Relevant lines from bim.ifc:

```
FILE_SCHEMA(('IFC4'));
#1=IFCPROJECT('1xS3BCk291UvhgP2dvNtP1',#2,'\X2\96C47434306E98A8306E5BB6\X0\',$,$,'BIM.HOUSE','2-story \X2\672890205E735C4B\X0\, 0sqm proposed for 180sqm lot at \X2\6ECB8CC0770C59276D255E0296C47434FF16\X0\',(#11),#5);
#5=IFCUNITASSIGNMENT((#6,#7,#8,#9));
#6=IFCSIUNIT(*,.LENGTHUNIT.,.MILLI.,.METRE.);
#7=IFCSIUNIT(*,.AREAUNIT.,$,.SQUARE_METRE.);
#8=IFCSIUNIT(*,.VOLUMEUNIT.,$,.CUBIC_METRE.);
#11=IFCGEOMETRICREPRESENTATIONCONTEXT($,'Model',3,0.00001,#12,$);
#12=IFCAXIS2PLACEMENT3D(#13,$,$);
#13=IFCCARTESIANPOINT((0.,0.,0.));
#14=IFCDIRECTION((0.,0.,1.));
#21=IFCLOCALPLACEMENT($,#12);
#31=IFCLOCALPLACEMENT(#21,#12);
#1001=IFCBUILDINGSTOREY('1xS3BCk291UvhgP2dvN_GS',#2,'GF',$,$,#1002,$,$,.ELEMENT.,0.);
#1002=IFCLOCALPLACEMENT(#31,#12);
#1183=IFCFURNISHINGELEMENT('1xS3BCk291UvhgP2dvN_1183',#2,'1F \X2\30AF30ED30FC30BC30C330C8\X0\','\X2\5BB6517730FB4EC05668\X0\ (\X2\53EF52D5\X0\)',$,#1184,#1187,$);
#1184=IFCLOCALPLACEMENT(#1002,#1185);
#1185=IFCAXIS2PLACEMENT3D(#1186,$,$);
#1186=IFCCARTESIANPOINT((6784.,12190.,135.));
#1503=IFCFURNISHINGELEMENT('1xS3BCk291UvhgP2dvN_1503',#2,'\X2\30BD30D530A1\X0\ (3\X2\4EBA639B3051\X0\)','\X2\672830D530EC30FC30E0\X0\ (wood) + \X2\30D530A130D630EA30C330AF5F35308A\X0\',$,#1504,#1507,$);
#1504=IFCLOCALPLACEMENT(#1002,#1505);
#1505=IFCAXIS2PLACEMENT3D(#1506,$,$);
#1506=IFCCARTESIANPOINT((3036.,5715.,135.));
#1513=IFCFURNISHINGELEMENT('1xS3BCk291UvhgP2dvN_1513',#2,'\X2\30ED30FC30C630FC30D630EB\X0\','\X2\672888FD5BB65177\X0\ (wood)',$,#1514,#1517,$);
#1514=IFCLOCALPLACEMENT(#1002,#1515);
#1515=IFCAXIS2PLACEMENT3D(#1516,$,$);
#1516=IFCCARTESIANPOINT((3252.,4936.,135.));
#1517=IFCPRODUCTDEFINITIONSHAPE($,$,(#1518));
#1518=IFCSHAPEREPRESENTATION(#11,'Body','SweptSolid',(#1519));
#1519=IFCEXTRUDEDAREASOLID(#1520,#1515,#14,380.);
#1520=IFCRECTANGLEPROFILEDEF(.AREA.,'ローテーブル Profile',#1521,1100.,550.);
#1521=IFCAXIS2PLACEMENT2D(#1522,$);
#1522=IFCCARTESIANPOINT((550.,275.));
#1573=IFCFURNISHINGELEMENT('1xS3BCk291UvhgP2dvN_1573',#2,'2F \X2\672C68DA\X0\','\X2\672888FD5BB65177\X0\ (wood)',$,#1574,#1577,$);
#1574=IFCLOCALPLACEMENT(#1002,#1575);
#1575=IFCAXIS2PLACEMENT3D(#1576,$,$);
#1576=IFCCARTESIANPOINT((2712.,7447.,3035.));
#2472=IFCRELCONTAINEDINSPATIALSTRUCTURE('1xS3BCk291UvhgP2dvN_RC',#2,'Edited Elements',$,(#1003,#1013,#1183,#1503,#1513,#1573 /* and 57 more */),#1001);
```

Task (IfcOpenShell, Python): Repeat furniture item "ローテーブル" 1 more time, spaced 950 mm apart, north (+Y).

```python
import numpy as np
import ifcopenshell
import ifcopenshell.api.geometry
import ifcopenshell.api.root
import ifcopenshell.util.element
import ifcopenshell.util.placement
import ifcopenshell.util.unit

model = ifcopenshell.open("bim.ifc")
unit_scale = ifcopenshell.util.unit.calculate_unit_scale(model)


def reuse_history(source, copy):
    """copy_class also copies each property set's owner history, people and application; keep the originals."""
    for rel in copy.IsDefinedBy:
        if rel.is_a("IfcRelDefinesByProperties") and (history := rel.RelatingPropertyDefinition.OwnerHistory):
            rel.RelatingPropertyDefinition.OwnerHistory = source.OwnerHistory
            ifcopenshell.util.element.remove_deep2(model, history)


source = model.by_guid("1xS3BCk291UvhgP2dvN_1513")
base = ifcopenshell.util.placement.get_local_placement(source.ObjectPlacement)
step = np.array([0.0, 1.0, 0.0]) * 0.95 / unit_scale

for i in range(1, 2):
    copy = ifcopenshell.api.root.copy_class(model, product=source)
    copy.Representation = ifcopenshell.util.element.copy_deep(
        model, source.Representation, exclude=["IfcGeometricRepresentationContext", "IfcRepresentationMap"]
    )
    reuse_history(source, copy)
    matrix = base.copy()
    matrix[:3, 3] += i * step
    print("added at", matrix[:3, 3].round(3) + 0.0)
    ifcopenshell.api.geometry.edit_object_placement(model, product=copy, matrix=matrix, is_si=False)

model.write("bim_rev.ifc")
```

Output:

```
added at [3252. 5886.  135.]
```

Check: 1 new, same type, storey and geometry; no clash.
